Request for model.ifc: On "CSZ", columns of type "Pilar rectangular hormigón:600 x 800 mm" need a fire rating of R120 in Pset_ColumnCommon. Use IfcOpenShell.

First a look at what the model holds.

```python
import ifcopenshell
import ifcopenshell.util.element

model = ifcopenshell.open("model.ifc")
print(model.schema)
storey = next(s for s in model.by_type("IfcBuildingStorey") if s.Name == "CSZ")
columns = [e for e in ifcopenshell.util.element.get_decomposition(storey) if e.is_a("IfcColumn")]
seen = {}
for e in columns:
    element_type = ifcopenshell.util.element.get_type(e)
    key = (element_type.Name if element_type != e and element_type else None, ifcopenshell.util.element.get_pset(e, "Pset_ColumnCommon", "FireRating"))
    seen[key] = seen.get(key, 0) + 1
for (name, value), count in sorted(seen.items(), key=str):
    print(count, "x", name, "|", value)
```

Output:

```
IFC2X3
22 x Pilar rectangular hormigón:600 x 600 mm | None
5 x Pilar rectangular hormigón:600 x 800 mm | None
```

```python
import ifcopenshell
import ifcopenshell.api.pset
import ifcopenshell.util.element

model = ifcopenshell.open("model.ifc")

storey = next(s for s in model.by_type("IfcBuildingStorey") if s.Name == "CSZ")
columns = [e for e in ifcopenshell.util.element.get_decomposition(storey) if e.is_a("IfcColumn")]

count = 0
for e in columns:
    element_type = ifcopenshell.util.element.get_type(e)
    if element_type in (None, e) or element_type.Name != "Pilar rectangular hormigón:600 x 800 mm":
        continue
    # add_pset returns the element's existing set when there is one.
    pset = ifcopenshell.api.pset.add_pset(model, product=e, name="Pset_ColumnCommon")
    ifcopenshell.api.pset.edit_pset(model, pset=pset, properties={"FireRating": "R120"})
    count += 1

print(count, "columns updated")

model.write("model-out.ifc")
```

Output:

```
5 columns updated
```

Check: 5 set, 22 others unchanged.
